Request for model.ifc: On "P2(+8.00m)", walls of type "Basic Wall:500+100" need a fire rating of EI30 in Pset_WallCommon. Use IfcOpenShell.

First a look at what the model holds.

```python
import ifcopenshell
import ifcopenshell.util.element

model = ifcopenshell.open("model.ifc")
print(model.schema)
storey = next(s for s in model.by_type("IfcBuildingStorey") if s.Name == "P2(+8.00m)")
walls = [e for e in ifcopenshell.util.element.get_decomposition(storey) if e.is_a("IfcWall")]
seen = {}
for e in walls:
    element_type = ifcopenshell.util.element.get_type(e)
    key = (element_type.Name if element_type != e and element_type else None, ifcopenshell.util.element.get_pset(e, "Pset_WallCommon", "FireRating"))
    seen[key] = seen.get(key, 0) + 1
for (name, value), count in sorted(seen.items(), key=str):
    print(count, "x", name, "|", value)
```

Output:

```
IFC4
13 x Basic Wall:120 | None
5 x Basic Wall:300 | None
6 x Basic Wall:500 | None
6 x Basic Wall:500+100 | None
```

```python
import ifcopenshell
import ifcopenshell.api.pset
import ifcopenshell.util.element

model = ifcopenshell.open("model.ifc")

storey = next(s for s in model.by_type("IfcBuildingStorey") if s.Name == "P2(+8.00m)")
walls = [e for e in ifcopenshell.util.element.get_decomposition(storey) if e.is_a("IfcWall")]

count = 0
for e in walls:
    element_type = ifcopenshell.util.element.get_type(e)
    if element_type in (None, e) or element_type.Name != "Basic Wall:500+100":
        continue
    # add_pset returns the element's existing set when there is one.
    pset = ifcopenshell.api.pset.add_pset(model, product=e, name="Pset_WallCommon")
    ifcopenshell.api.pset.edit_pset(model, pset=pset, properties={"FireRating": "EI30"})
    count += 1

print(count, "walls updated")

model.write("model_updated.ifc")
```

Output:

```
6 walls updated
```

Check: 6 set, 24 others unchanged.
